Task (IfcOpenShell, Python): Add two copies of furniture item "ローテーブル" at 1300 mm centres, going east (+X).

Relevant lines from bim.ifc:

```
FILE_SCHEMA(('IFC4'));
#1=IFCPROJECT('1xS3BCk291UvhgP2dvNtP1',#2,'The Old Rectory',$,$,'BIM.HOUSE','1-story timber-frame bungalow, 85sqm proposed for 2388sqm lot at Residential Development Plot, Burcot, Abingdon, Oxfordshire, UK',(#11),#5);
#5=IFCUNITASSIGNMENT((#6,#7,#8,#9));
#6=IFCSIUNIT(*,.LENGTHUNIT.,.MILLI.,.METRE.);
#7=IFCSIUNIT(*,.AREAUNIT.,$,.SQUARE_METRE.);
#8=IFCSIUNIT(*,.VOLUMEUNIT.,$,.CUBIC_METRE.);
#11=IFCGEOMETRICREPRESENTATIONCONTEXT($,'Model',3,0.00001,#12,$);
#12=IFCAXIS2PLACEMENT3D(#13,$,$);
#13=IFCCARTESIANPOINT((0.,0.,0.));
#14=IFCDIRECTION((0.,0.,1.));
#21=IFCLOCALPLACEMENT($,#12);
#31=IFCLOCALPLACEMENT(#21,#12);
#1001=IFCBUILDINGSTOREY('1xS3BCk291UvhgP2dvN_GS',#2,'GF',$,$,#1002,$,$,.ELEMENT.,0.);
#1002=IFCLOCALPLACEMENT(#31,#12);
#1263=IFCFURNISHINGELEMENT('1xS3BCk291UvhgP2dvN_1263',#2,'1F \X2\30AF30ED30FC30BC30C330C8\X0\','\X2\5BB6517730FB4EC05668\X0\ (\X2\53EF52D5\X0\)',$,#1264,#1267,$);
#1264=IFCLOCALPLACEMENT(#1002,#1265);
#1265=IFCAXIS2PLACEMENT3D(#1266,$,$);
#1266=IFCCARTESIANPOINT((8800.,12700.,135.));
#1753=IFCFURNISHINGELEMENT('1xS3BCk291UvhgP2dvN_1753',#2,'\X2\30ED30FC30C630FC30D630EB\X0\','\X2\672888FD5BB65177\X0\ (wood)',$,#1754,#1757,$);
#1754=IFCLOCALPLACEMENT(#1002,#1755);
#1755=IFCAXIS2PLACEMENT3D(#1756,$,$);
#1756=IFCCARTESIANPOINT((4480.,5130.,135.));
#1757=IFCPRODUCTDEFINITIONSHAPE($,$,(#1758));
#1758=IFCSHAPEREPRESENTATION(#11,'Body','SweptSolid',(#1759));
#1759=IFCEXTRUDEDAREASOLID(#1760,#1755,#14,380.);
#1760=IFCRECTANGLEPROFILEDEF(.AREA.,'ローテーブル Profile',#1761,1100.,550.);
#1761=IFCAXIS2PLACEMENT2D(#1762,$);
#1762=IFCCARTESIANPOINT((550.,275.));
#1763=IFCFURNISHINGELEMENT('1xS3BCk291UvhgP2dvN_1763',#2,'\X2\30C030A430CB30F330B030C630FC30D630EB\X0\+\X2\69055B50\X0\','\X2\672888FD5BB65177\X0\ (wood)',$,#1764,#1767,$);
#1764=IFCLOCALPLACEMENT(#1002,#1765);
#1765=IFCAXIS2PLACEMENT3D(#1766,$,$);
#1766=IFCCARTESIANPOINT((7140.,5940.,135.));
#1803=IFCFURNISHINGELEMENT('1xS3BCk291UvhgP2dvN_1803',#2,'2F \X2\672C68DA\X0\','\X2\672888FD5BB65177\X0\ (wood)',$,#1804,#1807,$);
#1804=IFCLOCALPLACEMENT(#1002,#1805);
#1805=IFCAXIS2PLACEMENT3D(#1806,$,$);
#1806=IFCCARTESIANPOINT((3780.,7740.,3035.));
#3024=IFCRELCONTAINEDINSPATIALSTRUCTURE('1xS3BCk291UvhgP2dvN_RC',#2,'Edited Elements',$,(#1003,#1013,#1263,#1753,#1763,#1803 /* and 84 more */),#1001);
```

```python
import numpy as np
import ifcopenshell
import ifcopenshell.api.geometry
import ifcopenshell.api.root
import ifcopenshell.util.element
import ifcopenshell.util.placement

model = ifcopenshell.open("bim.ifc")


def reuse_history(source, copy):
    """copy_class also copies each property set's owner history, people and application; keep the originals."""
    for rel in copy.IsDefinedBy:
        if rel.is_a("IfcRelDefinesByProperties") and (history := rel.RelatingPropertyDefinition.OwnerHistory):
            rel.RelatingPropertyDefinition.OwnerHistory = source.OwnerHistory
            ifcopenshell.util.element.remove_deep2(model, history)


source = model.by_guid("1xS3BCk291UvhgP2dvN_1753")
base = ifcopenshell.util.placement.get_local_placement(source.ObjectPlacement)
step = np.array([1.0, 0.0, 0.0]) * 1300.0

for i in range(1, 3):
    copy = ifcopenshell.api.root.copy_class(model, product=source)
    copy.Representation = ifcopenshell.util.element.copy_deep(
        model, source.Representation, exclude=["IfcGeometricRepresentationContext", "IfcRepresentationMap"]
    )
    reuse_history(source, copy)
    matrix = base.copy()
    matrix[:3, 3] += i * step
    print("added at", matrix[:3, 3].round(3) + 0.0)
    ifcopenshell.api.geometry.edit_object_placement(model, product=copy, matrix=matrix, is_si=False)

model.write("bim_edited.ifc")
```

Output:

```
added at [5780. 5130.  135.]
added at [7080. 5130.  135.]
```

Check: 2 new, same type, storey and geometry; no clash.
